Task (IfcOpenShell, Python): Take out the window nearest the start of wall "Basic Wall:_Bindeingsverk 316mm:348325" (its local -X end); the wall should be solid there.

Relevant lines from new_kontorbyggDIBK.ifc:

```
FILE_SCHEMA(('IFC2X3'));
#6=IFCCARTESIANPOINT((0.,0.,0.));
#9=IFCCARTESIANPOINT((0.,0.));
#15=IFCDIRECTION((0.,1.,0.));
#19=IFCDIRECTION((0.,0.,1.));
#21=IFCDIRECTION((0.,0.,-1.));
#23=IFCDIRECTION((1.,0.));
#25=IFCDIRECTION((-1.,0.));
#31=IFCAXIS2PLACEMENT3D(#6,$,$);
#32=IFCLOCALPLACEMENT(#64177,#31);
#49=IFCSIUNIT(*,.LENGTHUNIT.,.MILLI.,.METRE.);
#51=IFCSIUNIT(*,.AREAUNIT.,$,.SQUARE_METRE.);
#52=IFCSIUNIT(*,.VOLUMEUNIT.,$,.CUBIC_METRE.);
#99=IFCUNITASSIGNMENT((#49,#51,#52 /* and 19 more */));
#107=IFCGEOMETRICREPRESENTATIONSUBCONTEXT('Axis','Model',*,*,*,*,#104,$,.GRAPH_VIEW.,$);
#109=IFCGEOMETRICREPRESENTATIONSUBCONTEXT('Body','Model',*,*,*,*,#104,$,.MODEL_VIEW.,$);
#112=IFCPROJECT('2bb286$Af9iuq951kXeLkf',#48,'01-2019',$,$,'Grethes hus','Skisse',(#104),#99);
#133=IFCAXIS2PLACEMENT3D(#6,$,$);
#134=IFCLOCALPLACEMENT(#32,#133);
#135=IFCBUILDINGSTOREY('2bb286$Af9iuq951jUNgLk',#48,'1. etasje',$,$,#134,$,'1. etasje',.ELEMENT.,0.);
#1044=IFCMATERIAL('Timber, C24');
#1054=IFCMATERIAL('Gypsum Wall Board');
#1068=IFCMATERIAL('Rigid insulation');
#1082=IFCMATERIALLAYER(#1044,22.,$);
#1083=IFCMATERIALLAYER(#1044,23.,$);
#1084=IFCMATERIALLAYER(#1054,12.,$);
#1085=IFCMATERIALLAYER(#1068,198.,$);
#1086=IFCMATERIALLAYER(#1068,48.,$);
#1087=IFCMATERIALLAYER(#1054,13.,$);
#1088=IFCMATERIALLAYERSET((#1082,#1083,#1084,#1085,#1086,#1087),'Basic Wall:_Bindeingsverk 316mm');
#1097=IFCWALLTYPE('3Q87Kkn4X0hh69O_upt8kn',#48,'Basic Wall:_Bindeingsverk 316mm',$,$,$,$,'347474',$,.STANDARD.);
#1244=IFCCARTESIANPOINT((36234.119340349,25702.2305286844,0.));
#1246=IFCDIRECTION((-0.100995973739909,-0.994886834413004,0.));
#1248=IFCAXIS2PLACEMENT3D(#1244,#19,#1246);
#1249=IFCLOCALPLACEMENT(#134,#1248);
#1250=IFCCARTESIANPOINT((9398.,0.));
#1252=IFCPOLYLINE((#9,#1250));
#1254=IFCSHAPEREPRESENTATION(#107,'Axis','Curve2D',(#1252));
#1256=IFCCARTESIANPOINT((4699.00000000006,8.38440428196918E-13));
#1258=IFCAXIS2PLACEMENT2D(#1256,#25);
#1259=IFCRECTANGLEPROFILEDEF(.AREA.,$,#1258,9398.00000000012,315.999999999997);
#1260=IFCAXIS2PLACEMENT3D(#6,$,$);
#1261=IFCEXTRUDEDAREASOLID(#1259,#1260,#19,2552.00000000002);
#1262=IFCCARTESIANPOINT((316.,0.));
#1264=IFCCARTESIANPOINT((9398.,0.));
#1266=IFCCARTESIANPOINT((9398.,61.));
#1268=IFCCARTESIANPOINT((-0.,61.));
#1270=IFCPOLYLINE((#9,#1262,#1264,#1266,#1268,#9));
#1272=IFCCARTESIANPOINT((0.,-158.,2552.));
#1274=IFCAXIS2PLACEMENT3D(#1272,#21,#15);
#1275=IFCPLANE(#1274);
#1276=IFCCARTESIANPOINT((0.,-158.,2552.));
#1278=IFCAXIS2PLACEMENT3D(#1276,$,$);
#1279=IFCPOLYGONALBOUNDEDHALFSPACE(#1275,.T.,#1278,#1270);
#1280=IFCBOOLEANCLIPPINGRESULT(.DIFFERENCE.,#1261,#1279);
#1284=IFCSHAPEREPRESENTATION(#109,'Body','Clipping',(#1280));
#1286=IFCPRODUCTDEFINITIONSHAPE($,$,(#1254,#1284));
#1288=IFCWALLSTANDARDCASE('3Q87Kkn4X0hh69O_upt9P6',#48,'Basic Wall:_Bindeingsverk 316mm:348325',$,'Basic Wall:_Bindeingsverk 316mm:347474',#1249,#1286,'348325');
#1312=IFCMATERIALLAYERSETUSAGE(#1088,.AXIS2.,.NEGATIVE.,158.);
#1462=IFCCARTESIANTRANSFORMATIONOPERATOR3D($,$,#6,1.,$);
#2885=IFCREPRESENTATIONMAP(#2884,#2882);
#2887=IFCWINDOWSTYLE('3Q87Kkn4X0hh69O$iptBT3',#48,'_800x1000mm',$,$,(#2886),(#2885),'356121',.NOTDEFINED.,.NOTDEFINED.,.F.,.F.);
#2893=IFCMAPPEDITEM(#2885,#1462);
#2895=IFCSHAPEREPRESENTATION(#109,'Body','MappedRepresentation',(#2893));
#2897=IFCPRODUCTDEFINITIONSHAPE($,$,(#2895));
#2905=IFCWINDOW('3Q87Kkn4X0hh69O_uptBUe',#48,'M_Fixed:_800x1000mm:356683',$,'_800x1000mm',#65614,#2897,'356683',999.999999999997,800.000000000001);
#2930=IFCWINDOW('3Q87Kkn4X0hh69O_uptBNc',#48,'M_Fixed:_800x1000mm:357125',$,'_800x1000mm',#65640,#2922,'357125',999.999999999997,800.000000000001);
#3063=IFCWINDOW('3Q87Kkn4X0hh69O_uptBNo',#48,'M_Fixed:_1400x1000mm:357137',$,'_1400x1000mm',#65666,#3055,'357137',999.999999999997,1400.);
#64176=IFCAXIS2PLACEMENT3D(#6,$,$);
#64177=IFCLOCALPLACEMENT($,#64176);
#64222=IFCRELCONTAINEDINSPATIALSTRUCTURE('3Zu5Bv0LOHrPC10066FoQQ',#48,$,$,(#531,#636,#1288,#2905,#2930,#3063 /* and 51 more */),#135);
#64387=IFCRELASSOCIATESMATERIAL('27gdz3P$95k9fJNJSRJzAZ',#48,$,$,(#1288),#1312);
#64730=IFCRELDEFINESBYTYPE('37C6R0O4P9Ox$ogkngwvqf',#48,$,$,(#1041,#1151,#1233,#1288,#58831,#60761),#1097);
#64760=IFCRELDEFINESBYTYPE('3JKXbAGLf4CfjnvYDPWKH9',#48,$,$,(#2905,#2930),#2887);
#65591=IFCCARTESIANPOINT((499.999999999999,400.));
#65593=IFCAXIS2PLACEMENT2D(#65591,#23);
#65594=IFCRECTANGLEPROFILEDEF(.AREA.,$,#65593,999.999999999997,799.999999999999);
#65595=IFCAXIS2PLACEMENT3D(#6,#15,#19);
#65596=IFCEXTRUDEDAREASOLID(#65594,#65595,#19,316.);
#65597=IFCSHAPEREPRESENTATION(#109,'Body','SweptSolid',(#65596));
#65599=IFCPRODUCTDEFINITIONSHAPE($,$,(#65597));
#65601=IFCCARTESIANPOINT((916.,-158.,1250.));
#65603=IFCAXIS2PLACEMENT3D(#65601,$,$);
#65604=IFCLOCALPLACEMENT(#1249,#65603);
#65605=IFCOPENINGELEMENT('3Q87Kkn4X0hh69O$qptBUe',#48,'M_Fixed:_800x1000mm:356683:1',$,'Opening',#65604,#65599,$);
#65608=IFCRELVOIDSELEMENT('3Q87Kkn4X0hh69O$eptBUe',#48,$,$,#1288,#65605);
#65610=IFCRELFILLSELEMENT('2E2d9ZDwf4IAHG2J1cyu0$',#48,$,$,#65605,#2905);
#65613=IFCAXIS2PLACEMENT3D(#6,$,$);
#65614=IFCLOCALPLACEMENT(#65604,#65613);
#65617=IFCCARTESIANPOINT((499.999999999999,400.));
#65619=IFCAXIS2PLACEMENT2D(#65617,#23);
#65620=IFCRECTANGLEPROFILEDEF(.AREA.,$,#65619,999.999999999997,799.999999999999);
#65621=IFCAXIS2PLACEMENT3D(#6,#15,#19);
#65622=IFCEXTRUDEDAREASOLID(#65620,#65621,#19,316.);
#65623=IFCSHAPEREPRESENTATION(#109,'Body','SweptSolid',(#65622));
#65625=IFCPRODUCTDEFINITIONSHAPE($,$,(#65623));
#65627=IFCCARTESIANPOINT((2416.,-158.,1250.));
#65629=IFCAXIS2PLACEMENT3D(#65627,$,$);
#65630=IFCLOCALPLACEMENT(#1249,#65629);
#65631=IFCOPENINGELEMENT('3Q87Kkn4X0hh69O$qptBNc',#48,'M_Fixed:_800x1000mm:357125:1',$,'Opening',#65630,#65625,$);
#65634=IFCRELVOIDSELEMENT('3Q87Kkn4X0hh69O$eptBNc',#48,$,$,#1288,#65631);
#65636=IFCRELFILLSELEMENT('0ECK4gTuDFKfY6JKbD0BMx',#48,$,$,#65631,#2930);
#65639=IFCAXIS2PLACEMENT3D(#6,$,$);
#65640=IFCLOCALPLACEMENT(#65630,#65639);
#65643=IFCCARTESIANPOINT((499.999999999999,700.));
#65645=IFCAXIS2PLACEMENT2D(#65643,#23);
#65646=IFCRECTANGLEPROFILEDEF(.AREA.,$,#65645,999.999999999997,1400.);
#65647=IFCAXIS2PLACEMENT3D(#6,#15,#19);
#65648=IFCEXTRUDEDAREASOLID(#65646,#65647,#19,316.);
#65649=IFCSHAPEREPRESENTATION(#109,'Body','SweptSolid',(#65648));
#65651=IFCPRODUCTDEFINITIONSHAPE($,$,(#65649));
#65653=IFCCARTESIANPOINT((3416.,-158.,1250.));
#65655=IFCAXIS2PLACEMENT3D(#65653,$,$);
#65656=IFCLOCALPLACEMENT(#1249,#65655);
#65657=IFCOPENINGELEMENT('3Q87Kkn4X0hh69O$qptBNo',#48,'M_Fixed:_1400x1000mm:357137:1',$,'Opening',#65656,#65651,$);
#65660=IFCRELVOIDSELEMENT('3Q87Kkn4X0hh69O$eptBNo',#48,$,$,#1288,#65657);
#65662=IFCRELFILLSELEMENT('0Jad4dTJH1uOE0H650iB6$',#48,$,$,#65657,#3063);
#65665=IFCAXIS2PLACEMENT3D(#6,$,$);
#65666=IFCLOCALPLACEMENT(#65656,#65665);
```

```python
import ifcopenshell
import ifcopenshell.api.feature
import ifcopenshell.api.root
import ifcopenshell.geom
import ifcopenshell.util.shape

model = ifcopenshell.open("new_kontorbyggDIBK.ifc")
settings = ifcopenshell.geom.settings()


def volume(element):
    """Net volume in cubic metres, openings subtracted."""
    shape = ifcopenshell.geom.create_shape(settings, element)
    return ifcopenshell.util.shape.get_volume(shape.geometry)


window = model.by_guid("3Q87Kkn4X0hh69O_uptBUe")
opening = window.FillsVoids[0].RelatingOpeningElement
wall = opening.VoidsElements[0].RelatingBuildingElement
before = volume(wall)

ifcopenshell.api.root.remove_product(model, product=window)
ifcopenshell.api.feature.remove_feature(model, feature=opening)

after = volume(wall)

print(f"wall volume {before:.3f} -> {after:.3f} m3")

model.write("new_kontorbyggDIBK_updated.ifc")
```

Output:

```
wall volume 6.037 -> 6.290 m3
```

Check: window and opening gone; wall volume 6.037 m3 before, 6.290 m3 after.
